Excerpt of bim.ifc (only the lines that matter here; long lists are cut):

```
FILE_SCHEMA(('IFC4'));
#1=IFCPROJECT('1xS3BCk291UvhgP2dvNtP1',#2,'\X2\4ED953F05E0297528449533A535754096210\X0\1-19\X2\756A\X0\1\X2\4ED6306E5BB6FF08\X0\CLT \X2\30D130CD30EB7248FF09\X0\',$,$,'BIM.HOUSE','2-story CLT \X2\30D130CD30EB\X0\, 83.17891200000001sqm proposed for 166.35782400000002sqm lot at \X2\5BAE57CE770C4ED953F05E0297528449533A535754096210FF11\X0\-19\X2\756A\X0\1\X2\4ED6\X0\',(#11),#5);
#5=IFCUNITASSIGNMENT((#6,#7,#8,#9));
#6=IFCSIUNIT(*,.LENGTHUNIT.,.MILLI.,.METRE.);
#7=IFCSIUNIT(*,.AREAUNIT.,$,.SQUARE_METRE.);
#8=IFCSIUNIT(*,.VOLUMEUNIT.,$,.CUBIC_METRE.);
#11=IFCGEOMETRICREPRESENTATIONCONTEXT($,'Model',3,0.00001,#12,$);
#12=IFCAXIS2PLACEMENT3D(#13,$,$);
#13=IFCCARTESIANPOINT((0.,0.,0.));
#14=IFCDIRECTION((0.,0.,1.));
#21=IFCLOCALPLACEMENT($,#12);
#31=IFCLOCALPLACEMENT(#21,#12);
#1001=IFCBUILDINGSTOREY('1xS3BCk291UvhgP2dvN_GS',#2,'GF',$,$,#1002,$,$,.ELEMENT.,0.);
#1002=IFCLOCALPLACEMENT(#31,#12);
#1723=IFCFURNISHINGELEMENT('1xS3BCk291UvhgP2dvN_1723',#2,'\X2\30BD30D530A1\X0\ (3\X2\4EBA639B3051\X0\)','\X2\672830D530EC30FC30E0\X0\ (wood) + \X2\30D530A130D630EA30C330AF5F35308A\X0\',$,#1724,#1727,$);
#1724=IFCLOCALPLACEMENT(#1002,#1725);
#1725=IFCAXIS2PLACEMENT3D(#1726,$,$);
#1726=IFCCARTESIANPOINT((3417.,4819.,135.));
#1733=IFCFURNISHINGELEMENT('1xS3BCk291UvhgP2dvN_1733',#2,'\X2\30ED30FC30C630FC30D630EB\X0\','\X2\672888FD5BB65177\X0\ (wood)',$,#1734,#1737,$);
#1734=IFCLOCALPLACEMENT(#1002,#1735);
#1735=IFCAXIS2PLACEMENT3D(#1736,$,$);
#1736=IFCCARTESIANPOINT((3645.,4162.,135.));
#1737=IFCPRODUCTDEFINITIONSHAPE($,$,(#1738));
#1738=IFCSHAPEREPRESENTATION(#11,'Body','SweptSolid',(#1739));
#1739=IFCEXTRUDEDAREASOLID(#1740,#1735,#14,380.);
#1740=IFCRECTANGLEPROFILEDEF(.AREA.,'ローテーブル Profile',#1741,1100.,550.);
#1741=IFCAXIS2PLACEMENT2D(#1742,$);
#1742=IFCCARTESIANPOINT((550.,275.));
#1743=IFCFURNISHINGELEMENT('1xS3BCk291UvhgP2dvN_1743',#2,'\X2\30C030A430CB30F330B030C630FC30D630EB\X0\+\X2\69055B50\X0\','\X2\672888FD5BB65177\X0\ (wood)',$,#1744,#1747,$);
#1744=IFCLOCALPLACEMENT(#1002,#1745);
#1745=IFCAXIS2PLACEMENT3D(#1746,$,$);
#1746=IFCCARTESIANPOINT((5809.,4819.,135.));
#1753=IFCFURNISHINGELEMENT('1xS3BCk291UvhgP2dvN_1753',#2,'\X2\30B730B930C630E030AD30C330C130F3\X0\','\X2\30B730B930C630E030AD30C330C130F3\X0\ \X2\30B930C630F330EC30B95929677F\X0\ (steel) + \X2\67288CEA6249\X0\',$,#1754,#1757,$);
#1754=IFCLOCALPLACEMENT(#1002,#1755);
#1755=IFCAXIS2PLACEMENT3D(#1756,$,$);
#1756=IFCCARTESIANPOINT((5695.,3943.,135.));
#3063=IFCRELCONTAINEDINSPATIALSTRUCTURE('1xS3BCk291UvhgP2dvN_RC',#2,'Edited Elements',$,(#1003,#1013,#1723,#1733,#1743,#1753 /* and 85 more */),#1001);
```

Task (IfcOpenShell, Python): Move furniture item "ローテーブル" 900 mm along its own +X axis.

```python
import ifcopenshell
import ifcopenshell.api.geometry
import ifcopenshell.util.placement
import ifcopenshell.util.unit

model = ifcopenshell.open("bim.ifc")
unit_scale = ifcopenshell.util.unit.calculate_unit_scale(model)

item = model.by_guid("1xS3BCk291UvhgP2dvN_1733")
matrix = ifcopenshell.util.placement.get_local_placement(item.ObjectPlacement)
matrix[:3, 3] += matrix[:3, 0] * 0.9 / unit_scale
ifcopenshell.api.geometry.edit_object_placement(model, product=item, matrix=matrix, is_si=False)

print(ifcopenshell.util.placement.get_local_placement(item.ObjectPlacement).round(3) + 0.0)

model.write("bim_rev.ifc")
```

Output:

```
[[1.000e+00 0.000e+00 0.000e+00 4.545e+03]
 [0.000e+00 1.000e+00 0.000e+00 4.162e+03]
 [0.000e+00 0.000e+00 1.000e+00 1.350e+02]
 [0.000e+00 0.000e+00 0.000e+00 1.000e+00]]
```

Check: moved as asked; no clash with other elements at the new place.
